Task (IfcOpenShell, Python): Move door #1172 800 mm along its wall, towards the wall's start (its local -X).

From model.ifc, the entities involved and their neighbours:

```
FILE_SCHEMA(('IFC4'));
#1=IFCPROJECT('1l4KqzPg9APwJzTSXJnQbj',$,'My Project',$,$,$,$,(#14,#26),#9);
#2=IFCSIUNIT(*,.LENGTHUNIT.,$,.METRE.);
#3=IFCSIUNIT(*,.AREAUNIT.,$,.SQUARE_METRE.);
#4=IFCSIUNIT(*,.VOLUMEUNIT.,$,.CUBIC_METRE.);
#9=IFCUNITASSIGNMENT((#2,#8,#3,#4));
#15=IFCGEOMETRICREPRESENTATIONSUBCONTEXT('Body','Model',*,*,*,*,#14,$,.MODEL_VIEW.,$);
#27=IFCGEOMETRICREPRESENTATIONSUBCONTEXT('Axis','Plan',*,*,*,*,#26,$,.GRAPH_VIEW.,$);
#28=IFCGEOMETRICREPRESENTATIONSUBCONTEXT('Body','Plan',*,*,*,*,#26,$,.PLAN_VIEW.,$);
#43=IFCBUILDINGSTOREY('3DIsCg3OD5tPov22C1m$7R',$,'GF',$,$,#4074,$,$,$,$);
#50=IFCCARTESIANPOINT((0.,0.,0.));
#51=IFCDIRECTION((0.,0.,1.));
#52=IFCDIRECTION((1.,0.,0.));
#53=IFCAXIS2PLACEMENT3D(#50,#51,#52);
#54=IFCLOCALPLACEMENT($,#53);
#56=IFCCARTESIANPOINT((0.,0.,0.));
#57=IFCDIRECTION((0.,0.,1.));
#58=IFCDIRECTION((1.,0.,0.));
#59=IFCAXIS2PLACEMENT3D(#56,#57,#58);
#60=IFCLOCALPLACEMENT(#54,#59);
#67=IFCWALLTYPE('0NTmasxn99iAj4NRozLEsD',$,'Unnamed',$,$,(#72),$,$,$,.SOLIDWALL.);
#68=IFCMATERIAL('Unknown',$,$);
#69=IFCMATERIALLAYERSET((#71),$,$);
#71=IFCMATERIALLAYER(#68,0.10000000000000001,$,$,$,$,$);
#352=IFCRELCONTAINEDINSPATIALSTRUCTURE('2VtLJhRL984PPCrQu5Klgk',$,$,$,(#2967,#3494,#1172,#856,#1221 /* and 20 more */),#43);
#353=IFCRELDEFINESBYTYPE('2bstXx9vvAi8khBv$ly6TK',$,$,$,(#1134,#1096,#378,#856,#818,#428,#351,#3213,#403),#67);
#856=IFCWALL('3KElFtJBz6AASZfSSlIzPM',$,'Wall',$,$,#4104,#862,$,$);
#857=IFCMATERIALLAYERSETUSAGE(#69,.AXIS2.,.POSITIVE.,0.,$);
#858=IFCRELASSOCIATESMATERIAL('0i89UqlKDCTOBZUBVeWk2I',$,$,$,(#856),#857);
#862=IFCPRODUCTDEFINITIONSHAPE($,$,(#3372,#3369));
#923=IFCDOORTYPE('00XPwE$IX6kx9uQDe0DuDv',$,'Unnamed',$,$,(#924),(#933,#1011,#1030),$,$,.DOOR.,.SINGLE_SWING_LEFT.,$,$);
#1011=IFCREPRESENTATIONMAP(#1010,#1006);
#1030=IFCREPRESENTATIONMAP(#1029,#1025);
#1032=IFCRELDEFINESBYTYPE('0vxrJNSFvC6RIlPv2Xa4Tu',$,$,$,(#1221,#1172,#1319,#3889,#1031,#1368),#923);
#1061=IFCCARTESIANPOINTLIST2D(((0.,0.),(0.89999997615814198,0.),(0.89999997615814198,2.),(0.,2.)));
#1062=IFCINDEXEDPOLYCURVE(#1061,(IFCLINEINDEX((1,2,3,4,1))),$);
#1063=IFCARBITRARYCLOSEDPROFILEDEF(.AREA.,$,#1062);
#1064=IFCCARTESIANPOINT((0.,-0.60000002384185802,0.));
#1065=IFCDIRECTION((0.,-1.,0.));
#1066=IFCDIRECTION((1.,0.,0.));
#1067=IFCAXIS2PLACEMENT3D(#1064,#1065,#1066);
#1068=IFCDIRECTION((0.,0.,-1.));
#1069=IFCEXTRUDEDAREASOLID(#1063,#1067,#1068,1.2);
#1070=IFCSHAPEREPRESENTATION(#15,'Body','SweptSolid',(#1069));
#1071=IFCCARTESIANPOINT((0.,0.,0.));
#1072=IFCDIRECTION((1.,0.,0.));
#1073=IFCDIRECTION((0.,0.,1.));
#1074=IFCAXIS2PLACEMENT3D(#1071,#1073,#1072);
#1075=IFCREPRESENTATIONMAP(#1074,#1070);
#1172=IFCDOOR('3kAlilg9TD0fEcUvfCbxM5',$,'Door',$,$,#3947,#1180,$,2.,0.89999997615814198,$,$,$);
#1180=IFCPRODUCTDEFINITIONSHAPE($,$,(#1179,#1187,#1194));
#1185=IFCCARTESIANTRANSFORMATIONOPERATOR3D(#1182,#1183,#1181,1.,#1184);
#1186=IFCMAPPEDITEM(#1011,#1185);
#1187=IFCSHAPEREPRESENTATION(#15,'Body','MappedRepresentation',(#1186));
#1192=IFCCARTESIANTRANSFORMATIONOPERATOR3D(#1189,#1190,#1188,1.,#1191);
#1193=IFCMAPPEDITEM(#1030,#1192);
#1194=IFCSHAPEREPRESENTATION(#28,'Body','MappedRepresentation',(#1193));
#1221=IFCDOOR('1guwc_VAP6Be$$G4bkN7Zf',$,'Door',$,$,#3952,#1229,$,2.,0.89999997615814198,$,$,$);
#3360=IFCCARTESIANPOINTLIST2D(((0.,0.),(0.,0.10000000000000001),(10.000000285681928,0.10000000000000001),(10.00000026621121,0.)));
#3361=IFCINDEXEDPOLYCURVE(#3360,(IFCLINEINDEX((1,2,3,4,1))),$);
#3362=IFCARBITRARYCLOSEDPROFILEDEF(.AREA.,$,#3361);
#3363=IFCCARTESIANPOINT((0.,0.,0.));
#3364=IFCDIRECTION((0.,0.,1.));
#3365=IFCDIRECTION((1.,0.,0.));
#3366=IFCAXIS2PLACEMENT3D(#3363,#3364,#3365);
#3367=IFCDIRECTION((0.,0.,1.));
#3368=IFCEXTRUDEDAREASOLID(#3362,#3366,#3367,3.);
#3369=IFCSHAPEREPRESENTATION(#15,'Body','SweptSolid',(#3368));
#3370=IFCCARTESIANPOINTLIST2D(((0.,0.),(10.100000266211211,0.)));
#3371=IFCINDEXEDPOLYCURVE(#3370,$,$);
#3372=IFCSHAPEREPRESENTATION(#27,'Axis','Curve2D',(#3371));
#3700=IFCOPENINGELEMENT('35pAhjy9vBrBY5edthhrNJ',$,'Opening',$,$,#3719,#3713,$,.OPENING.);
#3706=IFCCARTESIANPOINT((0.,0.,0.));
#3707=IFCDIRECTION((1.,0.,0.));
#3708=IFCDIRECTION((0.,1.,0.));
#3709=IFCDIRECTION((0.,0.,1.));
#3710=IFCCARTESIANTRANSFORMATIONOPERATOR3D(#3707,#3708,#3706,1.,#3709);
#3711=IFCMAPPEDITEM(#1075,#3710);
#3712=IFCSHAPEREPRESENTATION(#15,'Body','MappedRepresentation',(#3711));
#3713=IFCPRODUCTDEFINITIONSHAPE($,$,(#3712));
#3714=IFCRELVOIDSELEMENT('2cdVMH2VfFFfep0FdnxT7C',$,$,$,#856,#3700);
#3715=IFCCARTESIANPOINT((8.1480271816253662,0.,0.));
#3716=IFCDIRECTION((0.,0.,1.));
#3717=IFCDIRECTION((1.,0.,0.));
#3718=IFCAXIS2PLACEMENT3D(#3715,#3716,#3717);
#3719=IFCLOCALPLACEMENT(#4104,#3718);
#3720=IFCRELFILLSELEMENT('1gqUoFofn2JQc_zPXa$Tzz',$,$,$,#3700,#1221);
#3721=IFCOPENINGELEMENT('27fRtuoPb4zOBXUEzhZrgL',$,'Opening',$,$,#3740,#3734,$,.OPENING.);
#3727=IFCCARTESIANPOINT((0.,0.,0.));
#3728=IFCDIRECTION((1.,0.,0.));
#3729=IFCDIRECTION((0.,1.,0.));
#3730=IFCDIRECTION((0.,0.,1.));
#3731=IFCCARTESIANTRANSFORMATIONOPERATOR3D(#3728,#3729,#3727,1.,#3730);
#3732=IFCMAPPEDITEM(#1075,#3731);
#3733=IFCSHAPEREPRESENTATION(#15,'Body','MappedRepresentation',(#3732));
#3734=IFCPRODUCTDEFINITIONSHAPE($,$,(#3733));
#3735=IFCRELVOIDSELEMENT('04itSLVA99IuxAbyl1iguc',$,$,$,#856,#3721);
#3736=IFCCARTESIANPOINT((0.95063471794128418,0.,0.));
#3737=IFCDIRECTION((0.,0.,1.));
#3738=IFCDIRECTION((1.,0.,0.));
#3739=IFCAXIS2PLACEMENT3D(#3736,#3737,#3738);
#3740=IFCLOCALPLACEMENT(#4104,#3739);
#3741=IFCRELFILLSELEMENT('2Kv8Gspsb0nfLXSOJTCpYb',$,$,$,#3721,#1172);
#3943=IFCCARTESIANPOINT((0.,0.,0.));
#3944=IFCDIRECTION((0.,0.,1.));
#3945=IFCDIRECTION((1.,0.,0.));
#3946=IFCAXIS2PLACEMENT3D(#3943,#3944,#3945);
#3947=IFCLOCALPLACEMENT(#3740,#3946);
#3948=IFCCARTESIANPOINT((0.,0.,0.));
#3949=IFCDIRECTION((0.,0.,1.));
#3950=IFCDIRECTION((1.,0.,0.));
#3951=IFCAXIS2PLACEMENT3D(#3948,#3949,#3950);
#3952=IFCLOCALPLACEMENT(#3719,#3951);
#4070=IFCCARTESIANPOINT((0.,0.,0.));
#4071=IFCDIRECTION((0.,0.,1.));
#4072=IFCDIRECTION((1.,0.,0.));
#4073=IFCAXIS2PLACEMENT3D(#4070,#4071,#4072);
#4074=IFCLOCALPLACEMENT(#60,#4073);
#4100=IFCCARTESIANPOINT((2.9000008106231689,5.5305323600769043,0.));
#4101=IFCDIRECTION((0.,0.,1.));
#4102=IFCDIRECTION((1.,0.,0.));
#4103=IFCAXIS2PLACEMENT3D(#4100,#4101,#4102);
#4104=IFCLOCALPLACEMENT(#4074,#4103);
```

```python
import ifcopenshell
import ifcopenshell.api.geometry
import ifcopenshell.util.placement

model = ifcopenshell.open("model.ifc")

door = model.by_guid("3kAlilg9TD0fEcUvfCbxM5")
opening = door.FillsVoids[0].RelatingOpeningElement
wall = opening.VoidsElements[0].RelatingBuildingElement

wall_matrix = ifcopenshell.util.placement.get_local_placement(wall.ObjectPlacement)
shift = wall_matrix[:3, 0] * -0.8
before = ifcopenshell.util.placement.get_local_placement(door.ObjectPlacement)[:3, 3].copy()

# The door is placed relative to its opening, so it follows when the opening moves.
matrix = ifcopenshell.util.placement.get_local_placement(opening.ObjectPlacement)
matrix[:3, 3] += shift
ifcopenshell.api.geometry.edit_object_placement(
    model, product=opening, matrix=matrix, is_si=False, should_transform_children=True
)

after = ifcopenshell.util.placement.get_local_placement(door.ObjectPlacement)[:3, 3]
print("door moved by", (after - before).round(3) + 0.0)

model.write("model-out.ifc")
```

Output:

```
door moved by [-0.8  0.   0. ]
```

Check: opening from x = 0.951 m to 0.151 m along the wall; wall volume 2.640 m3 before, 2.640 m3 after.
